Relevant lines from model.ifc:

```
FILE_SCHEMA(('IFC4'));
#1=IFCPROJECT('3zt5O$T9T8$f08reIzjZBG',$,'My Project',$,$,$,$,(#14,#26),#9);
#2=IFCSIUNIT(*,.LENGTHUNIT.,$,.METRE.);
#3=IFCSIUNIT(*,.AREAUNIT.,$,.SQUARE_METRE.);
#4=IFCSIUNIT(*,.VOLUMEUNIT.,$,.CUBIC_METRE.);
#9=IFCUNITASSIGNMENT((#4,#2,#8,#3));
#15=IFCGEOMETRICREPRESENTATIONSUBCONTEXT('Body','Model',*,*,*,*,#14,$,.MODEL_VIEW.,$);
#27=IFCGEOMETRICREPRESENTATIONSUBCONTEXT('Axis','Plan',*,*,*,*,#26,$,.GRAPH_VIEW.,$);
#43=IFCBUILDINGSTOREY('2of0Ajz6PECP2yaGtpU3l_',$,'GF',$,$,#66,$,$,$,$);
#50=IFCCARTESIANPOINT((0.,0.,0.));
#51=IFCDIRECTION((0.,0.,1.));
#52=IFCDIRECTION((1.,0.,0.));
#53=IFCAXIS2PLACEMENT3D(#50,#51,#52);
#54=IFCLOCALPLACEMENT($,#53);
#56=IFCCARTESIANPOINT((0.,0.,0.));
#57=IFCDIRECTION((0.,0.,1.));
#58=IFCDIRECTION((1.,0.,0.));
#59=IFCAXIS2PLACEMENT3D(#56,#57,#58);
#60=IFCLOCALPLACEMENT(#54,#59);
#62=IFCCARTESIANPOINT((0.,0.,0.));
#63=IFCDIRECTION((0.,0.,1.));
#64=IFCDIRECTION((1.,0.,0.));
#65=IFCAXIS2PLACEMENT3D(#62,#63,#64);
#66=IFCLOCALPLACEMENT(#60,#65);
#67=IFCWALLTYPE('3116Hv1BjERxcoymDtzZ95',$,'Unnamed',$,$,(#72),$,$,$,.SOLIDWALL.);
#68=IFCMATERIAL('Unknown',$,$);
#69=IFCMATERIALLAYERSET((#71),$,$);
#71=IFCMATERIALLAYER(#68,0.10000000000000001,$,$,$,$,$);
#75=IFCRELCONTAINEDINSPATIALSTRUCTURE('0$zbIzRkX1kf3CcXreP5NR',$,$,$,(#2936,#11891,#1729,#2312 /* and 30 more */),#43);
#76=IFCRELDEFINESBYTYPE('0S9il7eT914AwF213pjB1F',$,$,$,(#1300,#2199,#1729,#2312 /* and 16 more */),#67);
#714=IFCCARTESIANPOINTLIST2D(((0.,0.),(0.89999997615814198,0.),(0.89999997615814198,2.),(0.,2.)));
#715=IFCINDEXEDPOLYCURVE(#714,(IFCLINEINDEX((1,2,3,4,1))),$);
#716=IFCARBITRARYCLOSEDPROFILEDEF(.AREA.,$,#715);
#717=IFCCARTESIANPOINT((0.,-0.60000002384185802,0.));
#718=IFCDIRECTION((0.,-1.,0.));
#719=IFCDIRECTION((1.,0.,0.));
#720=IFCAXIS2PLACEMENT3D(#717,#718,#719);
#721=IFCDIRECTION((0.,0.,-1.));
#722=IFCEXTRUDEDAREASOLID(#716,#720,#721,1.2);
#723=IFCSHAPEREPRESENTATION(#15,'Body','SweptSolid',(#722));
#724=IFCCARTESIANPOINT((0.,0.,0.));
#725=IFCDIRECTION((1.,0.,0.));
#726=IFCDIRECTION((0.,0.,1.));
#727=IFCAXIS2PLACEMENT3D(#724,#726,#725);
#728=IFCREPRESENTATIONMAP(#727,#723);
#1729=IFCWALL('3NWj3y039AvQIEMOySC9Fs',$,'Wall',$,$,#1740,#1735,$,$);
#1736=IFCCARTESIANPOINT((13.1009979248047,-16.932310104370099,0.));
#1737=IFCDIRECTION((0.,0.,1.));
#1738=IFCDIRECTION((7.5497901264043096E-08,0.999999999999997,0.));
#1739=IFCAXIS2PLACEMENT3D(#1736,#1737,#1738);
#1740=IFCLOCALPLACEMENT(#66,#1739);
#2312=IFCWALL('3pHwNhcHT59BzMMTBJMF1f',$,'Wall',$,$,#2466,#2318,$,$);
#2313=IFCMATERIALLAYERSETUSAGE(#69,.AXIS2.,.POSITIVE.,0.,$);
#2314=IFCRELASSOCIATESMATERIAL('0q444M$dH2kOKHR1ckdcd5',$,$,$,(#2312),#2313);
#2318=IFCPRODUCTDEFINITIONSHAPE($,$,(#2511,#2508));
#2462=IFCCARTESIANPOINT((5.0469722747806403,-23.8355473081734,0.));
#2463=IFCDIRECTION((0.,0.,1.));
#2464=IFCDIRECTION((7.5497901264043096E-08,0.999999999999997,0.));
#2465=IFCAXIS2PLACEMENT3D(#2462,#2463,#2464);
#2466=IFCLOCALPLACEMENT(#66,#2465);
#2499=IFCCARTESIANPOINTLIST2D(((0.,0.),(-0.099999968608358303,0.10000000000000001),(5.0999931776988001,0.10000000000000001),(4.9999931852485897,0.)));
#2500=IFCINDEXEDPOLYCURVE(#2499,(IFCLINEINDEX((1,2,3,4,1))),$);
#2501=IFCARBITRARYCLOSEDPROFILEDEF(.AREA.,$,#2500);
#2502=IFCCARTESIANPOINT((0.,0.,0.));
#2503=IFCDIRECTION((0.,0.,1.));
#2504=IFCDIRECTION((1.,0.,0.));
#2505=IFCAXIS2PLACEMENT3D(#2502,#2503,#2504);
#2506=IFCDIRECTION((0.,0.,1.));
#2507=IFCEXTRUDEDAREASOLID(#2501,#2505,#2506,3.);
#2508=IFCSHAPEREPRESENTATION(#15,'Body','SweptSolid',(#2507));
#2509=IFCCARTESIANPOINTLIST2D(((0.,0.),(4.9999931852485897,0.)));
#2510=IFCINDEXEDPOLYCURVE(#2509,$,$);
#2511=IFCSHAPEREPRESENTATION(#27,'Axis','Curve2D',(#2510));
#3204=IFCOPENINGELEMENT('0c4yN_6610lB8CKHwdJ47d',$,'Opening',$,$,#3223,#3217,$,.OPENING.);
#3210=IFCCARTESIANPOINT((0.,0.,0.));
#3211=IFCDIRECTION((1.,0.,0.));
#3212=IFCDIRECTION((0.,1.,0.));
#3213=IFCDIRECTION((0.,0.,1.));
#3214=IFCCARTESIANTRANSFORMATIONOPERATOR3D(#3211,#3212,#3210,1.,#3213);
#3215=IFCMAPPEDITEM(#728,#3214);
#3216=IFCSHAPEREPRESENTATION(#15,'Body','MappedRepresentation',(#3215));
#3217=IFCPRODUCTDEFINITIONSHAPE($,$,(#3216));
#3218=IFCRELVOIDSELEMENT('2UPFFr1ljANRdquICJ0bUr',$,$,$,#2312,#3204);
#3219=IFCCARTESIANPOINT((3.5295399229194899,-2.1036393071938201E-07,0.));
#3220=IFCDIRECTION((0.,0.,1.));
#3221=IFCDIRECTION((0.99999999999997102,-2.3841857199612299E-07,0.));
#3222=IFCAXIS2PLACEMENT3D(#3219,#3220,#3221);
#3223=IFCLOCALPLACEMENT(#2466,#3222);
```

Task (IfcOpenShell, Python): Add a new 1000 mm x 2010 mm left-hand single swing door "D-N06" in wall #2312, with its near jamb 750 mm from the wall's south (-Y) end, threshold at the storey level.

```python
import numpy as np
import ifcopenshell
import ifcopenshell.api.feature
import ifcopenshell.api.geometry
import ifcopenshell.api.root
import ifcopenshell.api.spatial
import ifcopenshell.geom
import ifcopenshell.util.element
import ifcopenshell.util.placement
import ifcopenshell.util.representation
import ifcopenshell.util.shape
import ifcopenshell.util.unit

model = ifcopenshell.open("model.ifc")
unit_scale = ifcopenshell.util.unit.calculate_unit_scale(model)
settings = ifcopenshell.geom.settings()


def volume(element):
    """Net volume in cubic metres, openings subtracted."""
    shape = ifcopenshell.geom.create_shape(settings, element)
    return ifcopenshell.util.shape.get_volume(shape.geometry)


wall = model.by_guid("3pHwNhcHT59BzMMTBJMF1f")
storey = ifcopenshell.util.element.get_container(wall, ifc_class="IfcBuildingStorey")
context = ifcopenshell.util.representation.get_context(model, "Model", "Body", "MODEL_VIEW")
before = volume(wall)

width, height, from_end, sill = 1, 2.01, 0.75, 0.0  # metres

# The wall runs along its own X axis, and the end named is its -X end.
wall_shape = ifcopenshell.geom.create_shape(settings, wall)
x, y, z = ifcopenshell.util.shape.get_vertices(wall_shape.geometry).T
start = x.min() + from_end
face, thickness = float(y.min()), float(y.max() - y.min())
wall_matrix = ifcopenshell.util.placement.get_local_placement(wall.ObjectPlacement)
level = ifcopenshell.util.placement.get_local_placement(storey.ObjectPlacement)[2, 3]


def in_wall(x, y):
    """Placement at x, y metres in the wall's axes, at sill height."""
    matrix = wall_matrix.copy()
    matrix[:, 3] = wall_matrix @ np.array([x / unit_scale, y / unit_scale, 0.0, 1.0])
    matrix[2, 3] = level + sill / unit_scale
    return matrix


# Opening: a box that overshoots both wall faces by 50 mm.
opening = ifcopenshell.api.root.create_entity(model, ifc_class="IfcOpeningElement", predefined_type="OPENING")
box = ifcopenshell.api.geometry.add_wall_representation(
    model, context=context, length=width, height=height, thickness=thickness + 0.1
)
ifcopenshell.api.geometry.assign_representation(model, product=opening, representation=box)
ifcopenshell.api.geometry.edit_object_placement(model, product=opening, matrix=in_wall(start, face - 0.05), is_si=False)
ifcopenshell.api.feature.add_feature(model, feature=opening, element=wall)

door = ifcopenshell.api.root.create_entity(model, ifc_class="IfcDoor", name="D-N06", predefined_type="DOOR")
door.OverallWidth, door.OverallHeight = width / unit_scale, height / unit_scale
door.OperationType = "SINGLE_SWING_LEFT"
body = ifcopenshell.api.geometry.add_door_representation(
    model,
    context=context,
    overall_width=door.OverallWidth,
    overall_height=door.OverallHeight,
    operation_type="SINGLE_SWING_LEFT",
    lining_properties={"LiningDepth": thickness / unit_scale, "ThresholdDepth": thickness / unit_scale},
)
ifcopenshell.api.geometry.assign_representation(model, product=door, representation=body)
ifcopenshell.api.spatial.assign_container(model, products=[door], relating_structure=storey)
ifcopenshell.api.feature.add_filling(model, opening=opening, element=door)

# The lining spans the wall, so the door starts at the wall face.
ifcopenshell.api.geometry.edit_object_placement(model, product=door, matrix=in_wall(start, face), is_si=False)

after = volume(wall)

print(f"wall volume {before:.3f} -> {after:.3f} m3")

model.write("model_edited.ifc")
```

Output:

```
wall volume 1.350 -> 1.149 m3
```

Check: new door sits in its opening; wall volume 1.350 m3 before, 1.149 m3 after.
